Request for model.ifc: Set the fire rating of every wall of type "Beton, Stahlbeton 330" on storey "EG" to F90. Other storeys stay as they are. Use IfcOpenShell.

First a look at what the model holds.

```python
import ifcopenshell
import ifcopenshell.util.element

model = ifcopenshell.open("model.ifc")
print(model.schema)
storey = next(s for s in model.by_type("IfcBuildingStorey") if s.Name == "EG")
walls = [e for e in ifcopenshell.util.element.get_decomposition(storey) if e.is_a("IfcWall")]
seen = {}
for e in walls:
    element_type = ifcopenshell.util.element.get_type(e)
    key = (element_type.Name if element_type != e and element_type else None, ifcopenshell.util.element.get_pset(e, "Pset_WallCommon", "FireRating"))
    seen[key] = seen.get(key, 0) + 1
for (name, value), count in sorted(seen.items(), key=str):
    print(count, "x", name, "|", value)
```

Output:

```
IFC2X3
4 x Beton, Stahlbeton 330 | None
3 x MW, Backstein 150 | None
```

```python
import ifcopenshell
import ifcopenshell.api.pset
import ifcopenshell.util.element

model = ifcopenshell.open("model.ifc")

storey = next(s for s in model.by_type("IfcBuildingStorey") if s.Name == "EG")
walls = [e for e in ifcopenshell.util.element.get_decomposition(storey) if e.is_a("IfcWall")]

count = 0
for e in walls:
    element_type = ifcopenshell.util.element.get_type(e)
    if element_type in (None, e) or element_type.Name != "Beton, Stahlbeton 330":
        continue
    # add_pset returns the element's existing set when there is one.
    pset = ifcopenshell.api.pset.add_pset(model, product=e, name="Pset_WallCommon")
    ifcopenshell.api.pset.edit_pset(model, pset=pset, properties={"FireRating": "F90"})
    count += 1

print(count, "walls updated")

model.write("model_v2.ifc")
```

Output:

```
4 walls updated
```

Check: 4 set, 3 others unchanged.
